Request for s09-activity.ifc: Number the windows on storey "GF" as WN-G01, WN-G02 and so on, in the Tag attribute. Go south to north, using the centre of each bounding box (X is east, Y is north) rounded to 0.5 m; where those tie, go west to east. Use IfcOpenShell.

First a look at what the model holds.

```python
import ifcopenshell
import ifcopenshell.util.element
import ifcopenshell.util.placement

model = ifcopenshell.open("s09-activity.ifc")
print(model.schema)
storey = next(s for s in model.by_type("IfcBuildingStorey") if s.Name == "GF")
windows = [e for e in ifcopenshell.util.element.get_decomposition(storey) if e.is_a("IfcWindow")]
for e in sorted(windows, key=lambda e: e.id()):
    origin = ifcopenshell.util.placement.get_local_placement(e.ObjectPlacement)[:3, 3]
    print(e.id(), e.Tag, e.Name, origin.round(2) + 0.0, sep=" | ")
```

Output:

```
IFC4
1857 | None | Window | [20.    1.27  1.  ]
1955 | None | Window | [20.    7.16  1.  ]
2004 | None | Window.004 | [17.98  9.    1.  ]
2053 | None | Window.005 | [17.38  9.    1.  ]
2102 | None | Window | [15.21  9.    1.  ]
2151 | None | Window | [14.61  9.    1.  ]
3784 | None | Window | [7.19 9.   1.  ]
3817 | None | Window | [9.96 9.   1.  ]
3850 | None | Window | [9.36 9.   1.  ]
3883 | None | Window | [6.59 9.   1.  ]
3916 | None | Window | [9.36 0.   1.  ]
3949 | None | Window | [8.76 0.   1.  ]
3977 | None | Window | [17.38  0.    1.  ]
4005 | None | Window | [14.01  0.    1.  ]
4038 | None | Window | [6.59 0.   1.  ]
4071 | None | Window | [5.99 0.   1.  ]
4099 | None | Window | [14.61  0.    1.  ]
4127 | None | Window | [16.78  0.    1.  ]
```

```python
import ifcopenshell
import ifcopenshell.geom
import ifcopenshell.util.element
import ifcopenshell.util.shape

model = ifcopenshell.open("s09-activity.ifc")
settings = ifcopenshell.geom.settings()
settings.set("use-world-coords", True)


def centre(element):
    shape = ifcopenshell.geom.create_shape(settings, element)
    return ifcopenshell.util.shape.get_bbox_centroid(shape.geometry)


storey = next(s for s in model.by_type("IfcBuildingStorey") if s.Name == "GF")
windows = [e for e in ifcopenshell.util.element.get_decomposition(storey) if e.is_a("IfcWindow")]

# Insertion points can sit at a corner or the storey origin, so sort by the geometry (in metres).
centres = {e: centre(e) for e in windows}
windows.sort(key=lambda e: (round(centres[e][1] / 0.5), centres[e][0]))

for i, e in enumerate(windows, start=1):
    number = f"WN-G{i:02d}"
    e.Tag = number
    print(e.id(), number)

model.write("s09-activity_v2.ifc")
```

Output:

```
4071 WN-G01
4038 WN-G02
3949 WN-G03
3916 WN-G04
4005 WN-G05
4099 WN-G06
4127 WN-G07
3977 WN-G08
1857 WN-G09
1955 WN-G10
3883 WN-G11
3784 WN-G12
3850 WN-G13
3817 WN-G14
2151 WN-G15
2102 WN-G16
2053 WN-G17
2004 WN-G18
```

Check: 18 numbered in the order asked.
